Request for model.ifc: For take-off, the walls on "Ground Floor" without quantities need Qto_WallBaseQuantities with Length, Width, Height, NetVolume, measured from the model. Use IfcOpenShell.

First a look at what the model holds.

```python
import ifcopenshell
import ifcopenshell.util.element
import ifcopenshell.util.unit

model = ifcopenshell.open("model.ifc")
print(model.schema)
for unit_type in ("LENGTHUNIT", "AREAUNIT", "VOLUMEUNIT"):
    print(unit_type, ifcopenshell.util.unit.calculate_unit_scale(model, unit_type))
storey = next(s for s in model.by_type("IfcBuildingStorey") if s.Name == "Ground Floor")
walls = [e for e in ifcopenshell.util.element.get_decomposition(storey) if e.is_a("IfcWall")]
for e in sorted(walls, key=lambda e: e.id()):
    print(e.id(), e.is_a(), e.Name, list(ifcopenshell.util.element.get_psets(e, qtos_only=True)), sep=" | ")
```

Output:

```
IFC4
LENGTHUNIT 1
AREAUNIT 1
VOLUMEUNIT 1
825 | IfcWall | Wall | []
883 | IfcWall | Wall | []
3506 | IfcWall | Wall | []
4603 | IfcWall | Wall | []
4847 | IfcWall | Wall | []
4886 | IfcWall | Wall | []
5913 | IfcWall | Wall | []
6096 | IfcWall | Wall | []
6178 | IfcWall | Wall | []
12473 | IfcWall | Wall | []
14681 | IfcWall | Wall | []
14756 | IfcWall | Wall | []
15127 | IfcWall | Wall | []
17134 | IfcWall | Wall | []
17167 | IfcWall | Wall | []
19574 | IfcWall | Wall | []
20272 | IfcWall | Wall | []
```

```python
import ifcopenshell
import ifcopenshell.api.pset
import ifcopenshell.geom
import ifcopenshell.util.element
import ifcopenshell.util.shape
import ifcopenshell.util.unit

model = ifcopenshell.open("model.ifc")
unit_scale = ifcopenshell.util.unit.calculate_unit_scale(model)
volume_scale = ifcopenshell.util.unit.calculate_unit_scale(model, "VOLUMEUNIT")
settings = ifcopenshell.geom.settings()

storey = next(s for s in model.by_type("IfcBuildingStorey") if s.Name == "Ground Floor")
walls = [e for e in ifcopenshell.util.element.get_decomposition(storey) if e.is_a("IfcWall")]

for e in sorted(walls, key=lambda e: e.id()):
    if ifcopenshell.util.element.get_psets(e, qtos_only=True, should_inherit=False):
        continue
    # Geometry comes back in metres, in the element's own axes.
    shape = ifcopenshell.geom.create_shape(settings, e)
    values = {
        "Length": ifcopenshell.util.shape.get_x(shape.geometry) / unit_scale,
        "Width": ifcopenshell.util.shape.get_y(shape.geometry) / unit_scale,
        "Height": ifcopenshell.util.shape.get_z(shape.geometry) / unit_scale,
        "NetVolume": ifcopenshell.util.shape.get_volume(shape.geometry) / volume_scale,
    }
    qto = ifcopenshell.api.pset.add_qto(model, product=e, name="Qto_WallBaseQuantities")
    ifcopenshell.api.pset.edit_qto(model, qto=qto, properties=values)
    print(e.id(), {k: round(v, 3) for k, v in values.items()})

model.write("model-out.ifc")
```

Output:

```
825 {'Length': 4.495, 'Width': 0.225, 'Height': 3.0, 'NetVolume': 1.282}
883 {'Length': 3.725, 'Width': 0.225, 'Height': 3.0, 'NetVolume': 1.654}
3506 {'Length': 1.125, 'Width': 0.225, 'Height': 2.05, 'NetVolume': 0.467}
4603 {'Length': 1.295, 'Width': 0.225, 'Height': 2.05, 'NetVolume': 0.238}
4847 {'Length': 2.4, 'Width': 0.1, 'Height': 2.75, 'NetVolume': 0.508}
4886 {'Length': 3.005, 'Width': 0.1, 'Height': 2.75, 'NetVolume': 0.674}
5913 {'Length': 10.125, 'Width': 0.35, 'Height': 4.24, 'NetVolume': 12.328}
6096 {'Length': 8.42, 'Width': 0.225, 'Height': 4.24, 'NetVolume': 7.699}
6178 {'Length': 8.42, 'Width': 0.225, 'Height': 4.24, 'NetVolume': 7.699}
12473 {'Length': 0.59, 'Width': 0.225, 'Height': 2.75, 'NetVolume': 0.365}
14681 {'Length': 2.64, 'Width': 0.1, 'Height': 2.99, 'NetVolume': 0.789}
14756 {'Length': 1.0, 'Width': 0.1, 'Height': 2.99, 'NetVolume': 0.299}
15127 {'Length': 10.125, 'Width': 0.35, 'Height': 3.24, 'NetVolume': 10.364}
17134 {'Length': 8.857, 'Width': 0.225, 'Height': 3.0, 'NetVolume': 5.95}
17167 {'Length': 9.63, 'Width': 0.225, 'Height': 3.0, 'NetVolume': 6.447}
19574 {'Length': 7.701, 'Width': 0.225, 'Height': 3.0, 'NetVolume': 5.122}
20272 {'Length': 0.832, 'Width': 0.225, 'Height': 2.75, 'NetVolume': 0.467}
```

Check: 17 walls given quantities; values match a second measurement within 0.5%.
